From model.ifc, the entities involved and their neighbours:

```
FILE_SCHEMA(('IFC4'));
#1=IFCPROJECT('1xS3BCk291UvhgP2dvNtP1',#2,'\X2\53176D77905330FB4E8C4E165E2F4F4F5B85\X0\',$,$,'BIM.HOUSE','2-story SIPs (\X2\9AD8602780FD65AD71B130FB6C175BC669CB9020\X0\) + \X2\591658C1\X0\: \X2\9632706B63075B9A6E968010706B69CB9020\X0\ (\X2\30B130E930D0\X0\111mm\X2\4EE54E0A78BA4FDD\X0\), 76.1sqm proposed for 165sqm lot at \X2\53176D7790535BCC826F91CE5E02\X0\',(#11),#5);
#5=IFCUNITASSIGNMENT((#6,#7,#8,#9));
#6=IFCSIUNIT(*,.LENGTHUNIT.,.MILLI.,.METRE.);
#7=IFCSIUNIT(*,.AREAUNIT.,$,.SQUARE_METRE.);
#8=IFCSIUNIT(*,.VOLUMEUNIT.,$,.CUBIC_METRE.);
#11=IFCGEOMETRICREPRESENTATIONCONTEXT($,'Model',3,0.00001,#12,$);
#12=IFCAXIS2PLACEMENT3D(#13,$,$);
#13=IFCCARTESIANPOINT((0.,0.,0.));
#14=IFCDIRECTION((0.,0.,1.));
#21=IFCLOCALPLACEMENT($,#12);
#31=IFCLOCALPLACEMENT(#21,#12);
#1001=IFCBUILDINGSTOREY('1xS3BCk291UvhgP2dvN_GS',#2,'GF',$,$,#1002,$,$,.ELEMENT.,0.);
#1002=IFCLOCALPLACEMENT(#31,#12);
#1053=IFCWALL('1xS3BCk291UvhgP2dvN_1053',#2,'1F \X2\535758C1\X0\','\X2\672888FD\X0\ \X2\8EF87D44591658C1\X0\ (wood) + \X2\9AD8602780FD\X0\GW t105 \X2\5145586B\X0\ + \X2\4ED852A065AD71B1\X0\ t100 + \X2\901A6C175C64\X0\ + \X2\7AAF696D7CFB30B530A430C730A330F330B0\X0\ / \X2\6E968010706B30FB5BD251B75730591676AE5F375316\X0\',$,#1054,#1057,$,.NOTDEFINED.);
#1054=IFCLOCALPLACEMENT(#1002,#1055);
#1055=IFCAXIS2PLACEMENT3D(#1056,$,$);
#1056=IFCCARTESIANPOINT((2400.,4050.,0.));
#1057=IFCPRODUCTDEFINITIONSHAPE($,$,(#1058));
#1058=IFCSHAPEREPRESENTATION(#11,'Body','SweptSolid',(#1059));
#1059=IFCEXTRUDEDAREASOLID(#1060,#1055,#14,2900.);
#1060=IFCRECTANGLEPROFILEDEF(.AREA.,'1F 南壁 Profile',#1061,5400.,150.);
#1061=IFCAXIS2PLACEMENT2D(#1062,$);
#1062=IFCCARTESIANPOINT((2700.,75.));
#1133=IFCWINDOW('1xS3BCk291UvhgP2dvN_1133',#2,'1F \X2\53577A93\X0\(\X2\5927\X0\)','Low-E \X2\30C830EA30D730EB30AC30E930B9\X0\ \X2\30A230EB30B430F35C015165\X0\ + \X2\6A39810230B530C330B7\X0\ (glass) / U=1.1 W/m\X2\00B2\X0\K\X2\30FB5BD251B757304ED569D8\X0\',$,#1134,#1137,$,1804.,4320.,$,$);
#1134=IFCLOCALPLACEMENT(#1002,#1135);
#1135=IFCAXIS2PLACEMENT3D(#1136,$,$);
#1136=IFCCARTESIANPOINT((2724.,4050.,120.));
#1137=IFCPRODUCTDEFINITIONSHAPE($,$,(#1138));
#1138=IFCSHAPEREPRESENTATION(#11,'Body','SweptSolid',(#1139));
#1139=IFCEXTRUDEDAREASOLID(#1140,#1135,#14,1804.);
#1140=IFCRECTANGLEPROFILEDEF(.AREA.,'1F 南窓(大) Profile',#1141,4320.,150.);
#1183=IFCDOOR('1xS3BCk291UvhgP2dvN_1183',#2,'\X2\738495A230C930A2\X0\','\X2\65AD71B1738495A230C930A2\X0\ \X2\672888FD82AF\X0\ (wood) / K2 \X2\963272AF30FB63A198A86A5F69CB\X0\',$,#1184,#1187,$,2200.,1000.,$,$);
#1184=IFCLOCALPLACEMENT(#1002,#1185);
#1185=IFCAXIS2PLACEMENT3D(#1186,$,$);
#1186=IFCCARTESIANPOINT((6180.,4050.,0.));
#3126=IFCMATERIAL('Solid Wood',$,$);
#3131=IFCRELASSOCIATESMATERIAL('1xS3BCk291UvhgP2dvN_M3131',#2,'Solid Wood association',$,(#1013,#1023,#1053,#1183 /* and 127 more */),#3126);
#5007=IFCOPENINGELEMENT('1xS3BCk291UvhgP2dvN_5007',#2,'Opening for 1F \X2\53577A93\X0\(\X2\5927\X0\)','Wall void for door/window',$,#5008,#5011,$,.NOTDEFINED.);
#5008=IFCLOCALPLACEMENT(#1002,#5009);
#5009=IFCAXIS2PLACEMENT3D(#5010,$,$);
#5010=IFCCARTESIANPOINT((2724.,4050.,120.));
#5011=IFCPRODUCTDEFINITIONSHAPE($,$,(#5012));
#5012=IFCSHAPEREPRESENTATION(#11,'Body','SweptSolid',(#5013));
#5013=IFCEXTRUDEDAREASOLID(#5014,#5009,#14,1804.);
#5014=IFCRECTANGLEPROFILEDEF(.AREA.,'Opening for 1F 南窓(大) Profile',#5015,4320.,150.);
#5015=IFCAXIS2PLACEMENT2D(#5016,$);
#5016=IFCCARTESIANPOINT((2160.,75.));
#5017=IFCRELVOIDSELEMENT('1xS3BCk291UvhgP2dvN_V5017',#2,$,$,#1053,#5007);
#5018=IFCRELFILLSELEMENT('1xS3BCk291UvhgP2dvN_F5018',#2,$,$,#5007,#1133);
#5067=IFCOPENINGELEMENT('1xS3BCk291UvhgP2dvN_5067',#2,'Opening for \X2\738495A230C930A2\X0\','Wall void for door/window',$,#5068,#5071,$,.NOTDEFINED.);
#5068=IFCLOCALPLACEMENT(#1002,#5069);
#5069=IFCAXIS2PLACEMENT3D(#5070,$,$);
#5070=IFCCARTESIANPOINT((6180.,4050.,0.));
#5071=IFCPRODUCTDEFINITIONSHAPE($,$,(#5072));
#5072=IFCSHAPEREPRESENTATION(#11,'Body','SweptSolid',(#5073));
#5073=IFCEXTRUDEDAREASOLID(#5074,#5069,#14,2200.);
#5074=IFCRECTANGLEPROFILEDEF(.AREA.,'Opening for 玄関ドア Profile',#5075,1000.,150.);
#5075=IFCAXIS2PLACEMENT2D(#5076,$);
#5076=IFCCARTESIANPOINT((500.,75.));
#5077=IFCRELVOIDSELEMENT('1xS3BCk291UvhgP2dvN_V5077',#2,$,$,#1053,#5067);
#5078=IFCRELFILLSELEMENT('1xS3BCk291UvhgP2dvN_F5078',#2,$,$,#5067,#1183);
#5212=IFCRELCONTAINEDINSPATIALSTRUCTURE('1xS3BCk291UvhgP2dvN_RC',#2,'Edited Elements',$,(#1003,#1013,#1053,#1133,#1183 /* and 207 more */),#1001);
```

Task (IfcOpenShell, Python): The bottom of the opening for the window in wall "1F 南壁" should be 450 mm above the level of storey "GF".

```python
import numpy as np
import ifcopenshell
import ifcopenshell.api.geometry
import ifcopenshell.geom
import ifcopenshell.util.element
import ifcopenshell.util.placement
import ifcopenshell.util.shape
import ifcopenshell.util.unit

model = ifcopenshell.open("model.ifc")
unit_scale = ifcopenshell.util.unit.calculate_unit_scale(model)

window = model.by_guid("1xS3BCk291UvhgP2dvN_1133")
opening = window.FillsVoids[0].RelatingOpeningElement
storey = ifcopenshell.util.element.get_container(window, ifc_class="IfcBuildingStorey")
level = ifcopenshell.util.placement.get_local_placement(storey.ObjectPlacement)[2, 3]

# The opening's origin need not be at the sill, so measure its lowest point.
shape = ifcopenshell.geom.create_shape(ifcopenshell.geom.settings(), opening)
bottom = ifcopenshell.util.shape.get_shape_bottom_elevation(shape, shape.geometry) / unit_scale
dz = level + 450.0 - bottom

shift = np.array([0.0, 0.0, dz])
# The window is not placed relative to its opening, so move both.
for product in (opening, window):
    matrix = ifcopenshell.util.placement.get_local_placement(product.ObjectPlacement)
    matrix[:3, 3] += shift
    ifcopenshell.api.geometry.edit_object_placement(model, product=product, matrix=matrix, is_si=False)

print(f"moved by {dz * unit_scale:+.3f} m")

model.write("model-out.ifc")
```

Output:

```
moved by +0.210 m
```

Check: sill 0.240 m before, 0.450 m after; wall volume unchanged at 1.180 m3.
